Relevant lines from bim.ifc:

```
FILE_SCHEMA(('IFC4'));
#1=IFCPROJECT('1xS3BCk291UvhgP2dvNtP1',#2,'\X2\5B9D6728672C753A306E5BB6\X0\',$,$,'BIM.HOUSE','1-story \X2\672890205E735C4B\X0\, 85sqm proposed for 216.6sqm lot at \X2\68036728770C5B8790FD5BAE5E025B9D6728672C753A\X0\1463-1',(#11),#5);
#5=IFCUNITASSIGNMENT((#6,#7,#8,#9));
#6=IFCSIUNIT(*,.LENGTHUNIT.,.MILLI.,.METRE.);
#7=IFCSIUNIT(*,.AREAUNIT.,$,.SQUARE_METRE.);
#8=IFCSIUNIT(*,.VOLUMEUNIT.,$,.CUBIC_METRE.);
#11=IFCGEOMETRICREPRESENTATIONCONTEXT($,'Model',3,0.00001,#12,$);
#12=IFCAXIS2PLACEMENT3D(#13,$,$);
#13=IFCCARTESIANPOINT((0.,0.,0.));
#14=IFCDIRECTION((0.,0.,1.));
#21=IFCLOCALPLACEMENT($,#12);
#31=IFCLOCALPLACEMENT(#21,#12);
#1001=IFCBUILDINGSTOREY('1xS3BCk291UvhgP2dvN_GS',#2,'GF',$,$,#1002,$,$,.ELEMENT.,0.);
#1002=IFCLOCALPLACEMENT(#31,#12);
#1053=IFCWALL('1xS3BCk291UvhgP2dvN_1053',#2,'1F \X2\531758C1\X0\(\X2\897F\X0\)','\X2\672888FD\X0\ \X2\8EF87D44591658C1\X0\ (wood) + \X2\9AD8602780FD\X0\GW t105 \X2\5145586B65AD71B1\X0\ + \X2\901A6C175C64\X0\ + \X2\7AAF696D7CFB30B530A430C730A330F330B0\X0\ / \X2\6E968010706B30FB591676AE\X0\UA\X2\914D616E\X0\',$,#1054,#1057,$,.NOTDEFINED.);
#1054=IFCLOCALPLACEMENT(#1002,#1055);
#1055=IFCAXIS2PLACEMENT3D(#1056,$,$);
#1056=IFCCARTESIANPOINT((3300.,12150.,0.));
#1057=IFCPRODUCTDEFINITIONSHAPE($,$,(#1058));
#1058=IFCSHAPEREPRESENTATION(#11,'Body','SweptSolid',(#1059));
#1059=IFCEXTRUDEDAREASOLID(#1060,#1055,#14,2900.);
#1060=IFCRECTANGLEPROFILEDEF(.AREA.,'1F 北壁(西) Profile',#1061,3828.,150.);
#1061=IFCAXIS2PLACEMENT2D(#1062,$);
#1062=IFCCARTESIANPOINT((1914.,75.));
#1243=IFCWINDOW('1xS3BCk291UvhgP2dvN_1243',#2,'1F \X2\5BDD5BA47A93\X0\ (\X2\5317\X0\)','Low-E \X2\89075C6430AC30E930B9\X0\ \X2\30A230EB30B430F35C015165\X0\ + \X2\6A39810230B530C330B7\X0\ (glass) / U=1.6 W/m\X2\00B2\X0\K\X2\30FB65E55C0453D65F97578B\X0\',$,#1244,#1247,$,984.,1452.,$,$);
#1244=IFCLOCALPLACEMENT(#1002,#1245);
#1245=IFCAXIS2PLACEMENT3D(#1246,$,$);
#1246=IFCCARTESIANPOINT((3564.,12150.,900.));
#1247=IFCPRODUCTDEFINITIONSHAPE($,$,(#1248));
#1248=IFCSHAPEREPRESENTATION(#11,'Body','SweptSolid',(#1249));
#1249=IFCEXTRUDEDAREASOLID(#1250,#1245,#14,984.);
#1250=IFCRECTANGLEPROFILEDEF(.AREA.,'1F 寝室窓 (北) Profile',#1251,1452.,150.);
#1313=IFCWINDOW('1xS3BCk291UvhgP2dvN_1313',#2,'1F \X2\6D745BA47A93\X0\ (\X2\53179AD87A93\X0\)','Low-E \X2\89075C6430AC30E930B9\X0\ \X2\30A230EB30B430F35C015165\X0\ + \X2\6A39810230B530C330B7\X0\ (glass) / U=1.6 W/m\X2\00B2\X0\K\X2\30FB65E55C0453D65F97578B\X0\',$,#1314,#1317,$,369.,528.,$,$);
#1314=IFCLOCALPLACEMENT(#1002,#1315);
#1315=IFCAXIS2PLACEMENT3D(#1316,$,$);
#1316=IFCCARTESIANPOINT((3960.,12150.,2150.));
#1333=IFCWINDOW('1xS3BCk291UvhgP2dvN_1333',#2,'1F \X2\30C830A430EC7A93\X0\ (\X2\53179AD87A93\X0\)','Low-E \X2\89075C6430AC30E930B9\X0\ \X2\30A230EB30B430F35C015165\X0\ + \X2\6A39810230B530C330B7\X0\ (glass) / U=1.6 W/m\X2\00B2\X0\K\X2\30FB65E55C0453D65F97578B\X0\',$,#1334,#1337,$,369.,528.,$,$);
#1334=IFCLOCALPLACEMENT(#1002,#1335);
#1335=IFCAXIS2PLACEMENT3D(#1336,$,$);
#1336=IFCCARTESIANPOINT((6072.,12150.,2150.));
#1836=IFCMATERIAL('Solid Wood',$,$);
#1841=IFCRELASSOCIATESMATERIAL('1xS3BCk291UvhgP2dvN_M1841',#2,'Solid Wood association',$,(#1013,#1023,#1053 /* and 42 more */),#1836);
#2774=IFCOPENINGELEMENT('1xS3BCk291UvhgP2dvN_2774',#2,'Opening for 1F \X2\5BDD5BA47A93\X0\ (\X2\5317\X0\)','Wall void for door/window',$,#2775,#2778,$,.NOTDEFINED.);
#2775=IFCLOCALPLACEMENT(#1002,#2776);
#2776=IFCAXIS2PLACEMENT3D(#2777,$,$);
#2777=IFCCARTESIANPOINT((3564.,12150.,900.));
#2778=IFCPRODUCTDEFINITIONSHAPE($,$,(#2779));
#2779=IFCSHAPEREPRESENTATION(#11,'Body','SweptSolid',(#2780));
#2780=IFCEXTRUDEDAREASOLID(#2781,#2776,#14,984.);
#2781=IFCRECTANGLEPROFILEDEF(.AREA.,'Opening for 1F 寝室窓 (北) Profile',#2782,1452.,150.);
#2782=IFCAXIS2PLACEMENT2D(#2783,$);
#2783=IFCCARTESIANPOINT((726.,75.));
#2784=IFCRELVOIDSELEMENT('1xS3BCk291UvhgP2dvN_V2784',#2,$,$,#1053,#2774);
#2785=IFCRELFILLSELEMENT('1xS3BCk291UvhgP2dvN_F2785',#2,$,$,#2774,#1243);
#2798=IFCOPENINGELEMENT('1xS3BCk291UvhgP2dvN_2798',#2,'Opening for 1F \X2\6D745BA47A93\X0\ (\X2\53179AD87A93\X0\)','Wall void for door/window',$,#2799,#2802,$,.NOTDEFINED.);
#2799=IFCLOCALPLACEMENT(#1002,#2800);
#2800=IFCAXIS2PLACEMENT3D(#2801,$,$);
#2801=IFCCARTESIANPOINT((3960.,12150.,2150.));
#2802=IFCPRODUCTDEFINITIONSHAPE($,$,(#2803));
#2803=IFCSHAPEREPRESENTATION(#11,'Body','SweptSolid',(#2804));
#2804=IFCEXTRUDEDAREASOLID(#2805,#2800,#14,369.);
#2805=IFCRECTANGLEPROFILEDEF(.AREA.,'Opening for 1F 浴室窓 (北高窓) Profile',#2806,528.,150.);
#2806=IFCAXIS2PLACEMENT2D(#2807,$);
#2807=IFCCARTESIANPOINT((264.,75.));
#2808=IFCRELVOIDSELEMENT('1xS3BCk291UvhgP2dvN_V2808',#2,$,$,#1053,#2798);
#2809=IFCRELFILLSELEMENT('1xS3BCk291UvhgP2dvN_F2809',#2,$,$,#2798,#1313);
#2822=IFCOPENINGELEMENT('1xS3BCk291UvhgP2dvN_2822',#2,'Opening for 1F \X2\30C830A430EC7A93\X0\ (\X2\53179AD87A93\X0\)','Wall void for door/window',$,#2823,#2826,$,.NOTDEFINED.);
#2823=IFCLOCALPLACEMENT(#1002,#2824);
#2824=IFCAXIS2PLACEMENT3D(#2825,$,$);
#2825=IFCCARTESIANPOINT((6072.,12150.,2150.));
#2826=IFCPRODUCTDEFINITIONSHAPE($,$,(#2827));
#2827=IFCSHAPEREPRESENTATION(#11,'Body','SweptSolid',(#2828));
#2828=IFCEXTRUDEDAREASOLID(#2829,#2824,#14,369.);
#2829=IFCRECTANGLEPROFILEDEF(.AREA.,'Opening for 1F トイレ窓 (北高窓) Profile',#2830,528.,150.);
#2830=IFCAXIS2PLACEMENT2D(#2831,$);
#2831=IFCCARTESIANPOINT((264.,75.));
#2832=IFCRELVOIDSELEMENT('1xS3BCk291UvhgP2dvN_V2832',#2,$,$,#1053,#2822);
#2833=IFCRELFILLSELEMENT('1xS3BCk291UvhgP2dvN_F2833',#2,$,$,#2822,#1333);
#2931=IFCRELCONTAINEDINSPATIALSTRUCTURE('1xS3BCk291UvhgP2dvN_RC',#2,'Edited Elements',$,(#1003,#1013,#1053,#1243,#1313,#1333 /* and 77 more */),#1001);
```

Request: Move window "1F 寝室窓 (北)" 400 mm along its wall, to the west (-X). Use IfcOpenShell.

```python
import ifcopenshell
import ifcopenshell.api.geometry
import ifcopenshell.util.placement
import ifcopenshell.util.unit

model = ifcopenshell.open("bim.ifc")
unit_scale = ifcopenshell.util.unit.calculate_unit_scale(model)

window = model.by_id(1243)
opening = window.FillsVoids[0].RelatingOpeningElement
wall = opening.VoidsElements[0].RelatingBuildingElement

wall_matrix = ifcopenshell.util.placement.get_local_placement(wall.ObjectPlacement)
shift = wall_matrix[:3, 0] * -0.4 / unit_scale
before = ifcopenshell.util.placement.get_local_placement(window.ObjectPlacement)[:3, 3].copy()

# The window is not placed relative to its opening, so move both.
for product in (opening, window):
    matrix = ifcopenshell.util.placement.get_local_placement(product.ObjectPlacement)
    matrix[:3, 3] += shift
    ifcopenshell.api.geometry.edit_object_placement(model, product=product, matrix=matrix, is_si=False)

after = ifcopenshell.util.placement.get_local_placement(window.ObjectPlacement)[:3, 3]
print("window moved by", (after - before).round(3) + 0.0)

model.write("bim-out.ifc")
```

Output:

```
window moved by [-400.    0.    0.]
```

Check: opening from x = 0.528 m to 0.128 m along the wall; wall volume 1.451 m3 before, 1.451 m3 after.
